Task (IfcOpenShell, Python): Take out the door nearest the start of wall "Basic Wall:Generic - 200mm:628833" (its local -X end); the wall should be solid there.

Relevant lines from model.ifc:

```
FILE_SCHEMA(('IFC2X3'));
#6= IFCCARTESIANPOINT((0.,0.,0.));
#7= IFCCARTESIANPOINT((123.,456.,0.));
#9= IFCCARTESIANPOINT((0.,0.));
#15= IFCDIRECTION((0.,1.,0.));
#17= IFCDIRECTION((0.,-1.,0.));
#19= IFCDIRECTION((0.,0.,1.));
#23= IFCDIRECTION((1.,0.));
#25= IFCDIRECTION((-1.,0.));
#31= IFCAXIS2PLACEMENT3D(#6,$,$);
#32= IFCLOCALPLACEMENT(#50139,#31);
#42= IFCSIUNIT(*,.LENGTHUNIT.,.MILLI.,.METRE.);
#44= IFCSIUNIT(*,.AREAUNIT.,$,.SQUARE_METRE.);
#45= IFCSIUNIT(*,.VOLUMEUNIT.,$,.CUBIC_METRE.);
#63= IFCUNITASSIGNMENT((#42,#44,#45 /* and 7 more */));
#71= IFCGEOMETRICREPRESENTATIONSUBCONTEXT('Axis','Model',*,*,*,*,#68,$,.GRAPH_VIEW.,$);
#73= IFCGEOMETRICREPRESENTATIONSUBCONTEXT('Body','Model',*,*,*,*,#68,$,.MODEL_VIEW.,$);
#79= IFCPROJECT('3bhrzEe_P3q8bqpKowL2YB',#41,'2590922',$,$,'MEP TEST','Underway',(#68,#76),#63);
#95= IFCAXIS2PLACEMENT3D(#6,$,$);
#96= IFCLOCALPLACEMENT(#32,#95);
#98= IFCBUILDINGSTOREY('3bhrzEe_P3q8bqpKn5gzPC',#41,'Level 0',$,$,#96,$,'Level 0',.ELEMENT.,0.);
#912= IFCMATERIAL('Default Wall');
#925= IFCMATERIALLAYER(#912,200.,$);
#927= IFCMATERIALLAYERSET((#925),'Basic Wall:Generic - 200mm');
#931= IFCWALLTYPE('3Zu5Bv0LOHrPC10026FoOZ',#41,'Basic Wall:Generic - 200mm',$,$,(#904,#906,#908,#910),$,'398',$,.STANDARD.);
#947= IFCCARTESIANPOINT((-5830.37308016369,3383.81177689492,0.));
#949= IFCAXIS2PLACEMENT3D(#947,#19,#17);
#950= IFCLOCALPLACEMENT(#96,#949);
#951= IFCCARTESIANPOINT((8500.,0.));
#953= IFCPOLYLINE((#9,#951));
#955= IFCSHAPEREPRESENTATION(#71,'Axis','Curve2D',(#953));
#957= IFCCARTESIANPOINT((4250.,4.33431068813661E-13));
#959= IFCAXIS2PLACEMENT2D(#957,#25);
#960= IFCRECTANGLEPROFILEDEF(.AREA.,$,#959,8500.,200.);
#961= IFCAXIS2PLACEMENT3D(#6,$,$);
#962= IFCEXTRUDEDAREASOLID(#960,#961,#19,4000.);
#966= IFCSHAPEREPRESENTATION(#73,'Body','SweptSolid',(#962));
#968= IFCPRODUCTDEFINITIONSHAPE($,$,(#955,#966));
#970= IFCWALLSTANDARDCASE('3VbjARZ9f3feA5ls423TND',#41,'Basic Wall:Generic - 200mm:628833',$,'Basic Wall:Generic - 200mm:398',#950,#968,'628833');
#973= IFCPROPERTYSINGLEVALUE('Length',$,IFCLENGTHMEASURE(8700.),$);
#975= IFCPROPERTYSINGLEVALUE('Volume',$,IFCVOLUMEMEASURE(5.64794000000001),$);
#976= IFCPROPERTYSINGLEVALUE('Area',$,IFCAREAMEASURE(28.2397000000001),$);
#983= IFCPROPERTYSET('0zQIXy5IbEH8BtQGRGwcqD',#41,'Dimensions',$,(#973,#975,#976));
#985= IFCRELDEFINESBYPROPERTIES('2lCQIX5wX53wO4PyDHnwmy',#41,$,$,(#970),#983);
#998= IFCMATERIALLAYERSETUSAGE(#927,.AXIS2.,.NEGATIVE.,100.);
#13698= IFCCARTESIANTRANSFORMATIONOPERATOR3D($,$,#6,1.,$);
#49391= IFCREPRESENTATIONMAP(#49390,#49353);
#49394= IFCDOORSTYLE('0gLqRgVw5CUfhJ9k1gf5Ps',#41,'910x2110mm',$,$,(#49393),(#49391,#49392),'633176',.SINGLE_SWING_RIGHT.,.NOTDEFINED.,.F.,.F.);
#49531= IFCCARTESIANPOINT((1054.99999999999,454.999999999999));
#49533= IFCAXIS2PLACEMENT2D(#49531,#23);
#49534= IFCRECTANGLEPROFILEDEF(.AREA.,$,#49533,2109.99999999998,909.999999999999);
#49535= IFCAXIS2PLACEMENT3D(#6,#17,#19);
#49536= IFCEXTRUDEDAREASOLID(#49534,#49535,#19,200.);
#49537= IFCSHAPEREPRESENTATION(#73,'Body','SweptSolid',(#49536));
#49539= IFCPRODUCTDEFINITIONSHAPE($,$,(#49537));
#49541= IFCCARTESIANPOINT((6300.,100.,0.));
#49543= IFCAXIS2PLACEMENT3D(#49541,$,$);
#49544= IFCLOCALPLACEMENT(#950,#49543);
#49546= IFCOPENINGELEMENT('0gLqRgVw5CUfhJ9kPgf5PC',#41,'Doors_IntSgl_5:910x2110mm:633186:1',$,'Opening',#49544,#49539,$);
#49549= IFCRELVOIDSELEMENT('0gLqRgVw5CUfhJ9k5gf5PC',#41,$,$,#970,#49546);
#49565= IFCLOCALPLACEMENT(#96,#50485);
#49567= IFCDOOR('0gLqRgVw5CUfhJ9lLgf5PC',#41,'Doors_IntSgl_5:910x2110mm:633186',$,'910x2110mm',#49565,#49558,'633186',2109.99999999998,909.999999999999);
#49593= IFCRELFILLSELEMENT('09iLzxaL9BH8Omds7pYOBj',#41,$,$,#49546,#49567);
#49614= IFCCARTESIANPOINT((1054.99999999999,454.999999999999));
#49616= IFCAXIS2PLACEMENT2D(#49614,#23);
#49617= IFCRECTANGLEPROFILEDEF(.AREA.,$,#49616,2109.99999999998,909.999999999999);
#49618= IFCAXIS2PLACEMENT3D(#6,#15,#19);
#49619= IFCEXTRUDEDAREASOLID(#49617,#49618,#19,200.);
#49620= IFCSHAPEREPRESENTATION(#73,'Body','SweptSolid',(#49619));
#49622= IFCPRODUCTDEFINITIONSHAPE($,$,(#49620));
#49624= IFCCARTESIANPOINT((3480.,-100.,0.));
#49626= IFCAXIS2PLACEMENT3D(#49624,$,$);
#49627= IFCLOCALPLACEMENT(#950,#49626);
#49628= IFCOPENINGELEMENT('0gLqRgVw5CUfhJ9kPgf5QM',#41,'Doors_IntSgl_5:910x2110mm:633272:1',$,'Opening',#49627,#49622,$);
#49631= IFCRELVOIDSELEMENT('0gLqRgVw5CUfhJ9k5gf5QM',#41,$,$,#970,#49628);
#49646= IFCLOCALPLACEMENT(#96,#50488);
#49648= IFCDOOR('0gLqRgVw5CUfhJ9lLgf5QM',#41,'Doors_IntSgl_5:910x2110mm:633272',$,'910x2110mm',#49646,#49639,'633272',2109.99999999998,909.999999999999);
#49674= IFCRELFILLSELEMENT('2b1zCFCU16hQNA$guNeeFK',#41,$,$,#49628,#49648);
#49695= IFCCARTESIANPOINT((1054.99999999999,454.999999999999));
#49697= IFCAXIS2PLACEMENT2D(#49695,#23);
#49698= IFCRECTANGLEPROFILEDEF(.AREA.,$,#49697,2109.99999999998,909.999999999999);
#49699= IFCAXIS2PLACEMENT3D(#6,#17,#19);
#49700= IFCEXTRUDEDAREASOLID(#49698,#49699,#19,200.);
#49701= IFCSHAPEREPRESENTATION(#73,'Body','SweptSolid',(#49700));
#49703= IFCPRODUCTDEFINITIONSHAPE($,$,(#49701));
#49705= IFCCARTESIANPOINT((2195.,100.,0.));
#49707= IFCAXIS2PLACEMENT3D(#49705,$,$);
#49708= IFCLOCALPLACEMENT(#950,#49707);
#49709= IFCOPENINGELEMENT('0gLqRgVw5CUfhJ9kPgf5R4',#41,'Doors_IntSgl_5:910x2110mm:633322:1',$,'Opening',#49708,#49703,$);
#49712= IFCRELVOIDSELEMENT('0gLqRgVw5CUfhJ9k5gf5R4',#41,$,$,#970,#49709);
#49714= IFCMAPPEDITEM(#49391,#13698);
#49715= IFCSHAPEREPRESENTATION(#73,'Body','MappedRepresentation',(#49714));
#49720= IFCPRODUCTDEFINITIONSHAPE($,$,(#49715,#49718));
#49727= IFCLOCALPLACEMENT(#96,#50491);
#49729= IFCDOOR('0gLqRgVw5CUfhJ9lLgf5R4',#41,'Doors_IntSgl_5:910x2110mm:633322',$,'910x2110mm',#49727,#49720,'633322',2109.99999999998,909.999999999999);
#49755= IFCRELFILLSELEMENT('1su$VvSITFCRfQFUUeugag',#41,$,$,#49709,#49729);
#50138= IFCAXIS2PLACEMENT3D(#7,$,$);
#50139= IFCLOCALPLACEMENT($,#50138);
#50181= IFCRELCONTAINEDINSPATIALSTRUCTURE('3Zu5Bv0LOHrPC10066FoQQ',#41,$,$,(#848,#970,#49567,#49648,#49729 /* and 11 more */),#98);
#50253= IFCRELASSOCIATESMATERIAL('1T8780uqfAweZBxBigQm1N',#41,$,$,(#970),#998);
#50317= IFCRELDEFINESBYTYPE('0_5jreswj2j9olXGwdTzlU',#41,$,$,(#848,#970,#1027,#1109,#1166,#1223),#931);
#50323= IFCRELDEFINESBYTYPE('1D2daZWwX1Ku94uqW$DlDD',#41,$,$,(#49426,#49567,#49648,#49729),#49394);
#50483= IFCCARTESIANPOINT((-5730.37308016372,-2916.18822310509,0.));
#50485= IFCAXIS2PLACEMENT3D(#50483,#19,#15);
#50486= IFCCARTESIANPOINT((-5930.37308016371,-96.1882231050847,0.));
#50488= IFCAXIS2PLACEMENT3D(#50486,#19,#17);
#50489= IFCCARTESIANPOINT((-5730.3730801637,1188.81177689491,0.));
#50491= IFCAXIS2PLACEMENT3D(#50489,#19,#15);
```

```python
import ifcopenshell
import ifcopenshell.api.feature
import ifcopenshell.api.pset
import ifcopenshell.api.root
import ifcopenshell.geom
import ifcopenshell.util.element
import ifcopenshell.util.shape
import ifcopenshell.util.unit

model = ifcopenshell.open("model.ifc")
area_scale = ifcopenshell.util.unit.calculate_unit_scale(model, "AREAUNIT")
volume_scale = ifcopenshell.util.unit.calculate_unit_scale(model, "VOLUMEUNIT")
settings = ifcopenshell.geom.settings()


def volume(element):
    """Net volume in cubic metres, openings subtracted."""
    shape = ifcopenshell.geom.create_shape(settings, element)
    return ifcopenshell.util.shape.get_volume(shape.geometry)


door = model.by_guid("0gLqRgVw5CUfhJ9lLgf5R4")
opening = door.FillsVoids[0].RelatingOpeningElement
wall = opening.VoidsElements[0].RelatingBuildingElement
before = volume(wall)

ifcopenshell.api.root.remove_product(model, product=door)
ifcopenshell.api.feature.remove_feature(model, feature=opening)

after = volume(wall)
thickness = 0.2  # wall thickness in metres

# Update the wall's stored quantities.
pset = model.by_id(ifcopenshell.util.element.get_pset(wall, "Dimensions", should_inherit=False)["id"])
ifcopenshell.api.pset.edit_pset(model, pset=pset, properties={
    "Volume": model.create_entity("IfcVolumeMeasure", after / volume_scale),
    "Area": model.create_entity("IfcAreaMeasure", after / thickness / area_scale),
})

print(f"wall volume {before:.3f} -> {after:.3f} m3")

model.write("model_rev.ifc")
```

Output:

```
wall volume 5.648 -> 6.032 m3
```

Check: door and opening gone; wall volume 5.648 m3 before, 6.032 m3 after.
